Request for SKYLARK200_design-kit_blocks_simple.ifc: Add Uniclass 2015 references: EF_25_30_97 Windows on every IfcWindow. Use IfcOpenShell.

First a look at what the model holds.

```python
import ifcopenshell

model = ifcopenshell.open("SKYLARK200_design-kit_blocks_simple.ifc")
print(model.schema)
print("classifications:", [c.Name for c in model.by_type("IfcClassification")])
for ifc_class in ("IfcDoor", "IfcRoof", "IfcStair", "IfcWall", "IfcWindow"):
    print(ifc_class, len(model.by_type(ifc_class)))
```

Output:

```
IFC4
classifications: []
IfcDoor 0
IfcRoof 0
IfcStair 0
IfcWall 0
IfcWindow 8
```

```python
import ifcopenshell
import ifcopenshell.api.classification

model = ifcopenshell.open("SKYLARK200_design-kit_blocks_simple.ifc")

system = ifcopenshell.api.classification.add_classification(model, classification="Uniclass 2015")

codes = {
    "IfcWindow": ("EF_25_30_97", "Windows"),
}
for ifc_class, (code, name) in codes.items():
    products = model.by_type(ifc_class)
    ifcopenshell.api.classification.add_reference(
        model, products=products, classification=system, identification=code, name=name
    )
    print(code, len(products))

model.write("SKYLARK200_design-kit_blocks_simple_rev.ifc")
```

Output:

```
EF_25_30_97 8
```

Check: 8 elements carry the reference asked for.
